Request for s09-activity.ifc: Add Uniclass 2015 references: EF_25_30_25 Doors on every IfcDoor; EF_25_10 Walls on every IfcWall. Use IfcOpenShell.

First a look at what the model holds.

```python
import ifcopenshell

model = ifcopenshell.open("s09-activity.ifc")
print(model.schema)
print("classifications:", [c.Name for c in model.by_type("IfcClassification")])
for ifc_class in ("IfcDoor", "IfcRoof", "IfcStair", "IfcWall", "IfcWindow"):
    print(ifc_class, len(model.by_type(ifc_class)))
```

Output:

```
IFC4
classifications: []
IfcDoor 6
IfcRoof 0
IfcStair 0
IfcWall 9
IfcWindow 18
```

```python
import ifcopenshell
import ifcopenshell.api.classification

model = ifcopenshell.open("s09-activity.ifc")

system = ifcopenshell.api.classification.add_classification(model, classification="Uniclass 2015")

codes = {
    "IfcDoor": ("EF_25_30_25", "Doors"),
    "IfcWall": ("EF_25_10", "Walls"),
}
for ifc_class, (code, name) in codes.items():
    products = model.by_type(ifc_class)
    ifcopenshell.api.classification.add_reference(
        model, products=products, classification=system, identification=code, name=name
    )
    print(code, len(products))

model.write("s09-activity-out.ifc")
```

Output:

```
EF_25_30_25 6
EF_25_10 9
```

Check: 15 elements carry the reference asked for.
